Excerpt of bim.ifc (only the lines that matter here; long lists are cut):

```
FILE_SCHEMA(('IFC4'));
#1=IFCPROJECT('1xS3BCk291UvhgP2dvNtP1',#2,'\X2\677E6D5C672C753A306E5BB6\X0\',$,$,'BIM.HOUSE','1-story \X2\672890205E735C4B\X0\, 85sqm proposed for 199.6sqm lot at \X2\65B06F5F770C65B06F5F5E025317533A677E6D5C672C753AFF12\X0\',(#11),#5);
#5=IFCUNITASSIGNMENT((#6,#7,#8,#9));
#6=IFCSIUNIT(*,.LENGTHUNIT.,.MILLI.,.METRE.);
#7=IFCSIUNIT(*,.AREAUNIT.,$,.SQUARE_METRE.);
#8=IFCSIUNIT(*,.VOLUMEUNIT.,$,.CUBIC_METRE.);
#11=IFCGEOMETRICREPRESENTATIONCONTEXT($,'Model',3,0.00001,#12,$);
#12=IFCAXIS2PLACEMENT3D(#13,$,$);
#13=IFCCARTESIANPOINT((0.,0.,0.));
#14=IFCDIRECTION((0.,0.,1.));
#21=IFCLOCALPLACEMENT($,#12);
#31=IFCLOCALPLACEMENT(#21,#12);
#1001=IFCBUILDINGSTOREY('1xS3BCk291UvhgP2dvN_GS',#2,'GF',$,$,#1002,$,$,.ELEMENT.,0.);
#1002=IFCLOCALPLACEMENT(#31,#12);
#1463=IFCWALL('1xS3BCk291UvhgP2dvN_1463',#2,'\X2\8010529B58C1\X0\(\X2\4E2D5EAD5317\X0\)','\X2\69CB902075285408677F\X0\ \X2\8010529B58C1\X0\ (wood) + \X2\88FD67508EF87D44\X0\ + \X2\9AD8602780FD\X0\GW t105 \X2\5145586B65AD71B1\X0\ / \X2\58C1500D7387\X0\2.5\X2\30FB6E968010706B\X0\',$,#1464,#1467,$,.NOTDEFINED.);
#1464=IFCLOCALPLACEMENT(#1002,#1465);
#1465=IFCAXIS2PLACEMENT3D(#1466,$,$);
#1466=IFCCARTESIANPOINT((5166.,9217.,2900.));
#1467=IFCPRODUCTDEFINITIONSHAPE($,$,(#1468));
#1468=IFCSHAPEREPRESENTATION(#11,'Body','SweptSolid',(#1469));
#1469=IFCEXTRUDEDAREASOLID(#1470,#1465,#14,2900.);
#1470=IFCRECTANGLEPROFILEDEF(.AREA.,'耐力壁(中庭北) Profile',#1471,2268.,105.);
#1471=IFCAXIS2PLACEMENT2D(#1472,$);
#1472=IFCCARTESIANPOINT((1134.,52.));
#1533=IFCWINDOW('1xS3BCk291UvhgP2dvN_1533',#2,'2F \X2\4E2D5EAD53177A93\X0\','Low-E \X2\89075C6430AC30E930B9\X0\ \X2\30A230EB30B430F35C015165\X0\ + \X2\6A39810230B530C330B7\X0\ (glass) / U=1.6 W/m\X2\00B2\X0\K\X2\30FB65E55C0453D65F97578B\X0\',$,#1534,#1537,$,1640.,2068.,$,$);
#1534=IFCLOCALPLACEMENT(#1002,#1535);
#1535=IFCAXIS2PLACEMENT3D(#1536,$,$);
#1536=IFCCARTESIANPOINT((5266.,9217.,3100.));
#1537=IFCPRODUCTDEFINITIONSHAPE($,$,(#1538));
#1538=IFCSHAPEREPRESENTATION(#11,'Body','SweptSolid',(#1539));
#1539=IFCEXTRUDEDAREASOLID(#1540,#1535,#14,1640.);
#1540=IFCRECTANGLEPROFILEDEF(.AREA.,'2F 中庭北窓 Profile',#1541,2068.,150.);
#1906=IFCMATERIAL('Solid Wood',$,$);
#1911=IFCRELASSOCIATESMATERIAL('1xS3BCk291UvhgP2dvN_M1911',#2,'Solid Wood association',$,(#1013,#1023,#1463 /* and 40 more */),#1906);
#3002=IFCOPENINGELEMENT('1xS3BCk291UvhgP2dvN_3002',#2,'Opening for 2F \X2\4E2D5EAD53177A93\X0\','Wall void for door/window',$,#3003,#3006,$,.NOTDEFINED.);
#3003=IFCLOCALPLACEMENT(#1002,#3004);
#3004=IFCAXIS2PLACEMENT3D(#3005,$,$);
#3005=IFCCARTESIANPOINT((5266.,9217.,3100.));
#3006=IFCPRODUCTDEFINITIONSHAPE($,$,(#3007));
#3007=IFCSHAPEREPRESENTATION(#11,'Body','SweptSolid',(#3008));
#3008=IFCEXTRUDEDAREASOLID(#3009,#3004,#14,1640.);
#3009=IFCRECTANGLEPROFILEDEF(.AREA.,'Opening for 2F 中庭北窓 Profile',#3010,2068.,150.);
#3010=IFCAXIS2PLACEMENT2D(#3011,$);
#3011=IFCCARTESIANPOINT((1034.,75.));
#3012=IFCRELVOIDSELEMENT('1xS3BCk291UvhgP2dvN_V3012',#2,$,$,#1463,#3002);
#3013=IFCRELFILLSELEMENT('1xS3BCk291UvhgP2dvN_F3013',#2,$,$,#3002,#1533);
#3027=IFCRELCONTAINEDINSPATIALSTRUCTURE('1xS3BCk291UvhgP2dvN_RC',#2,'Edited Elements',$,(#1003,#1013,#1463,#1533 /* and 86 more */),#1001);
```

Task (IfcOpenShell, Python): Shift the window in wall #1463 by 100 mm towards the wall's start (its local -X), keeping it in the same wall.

```python
import ifcopenshell
import ifcopenshell.api.geometry
import ifcopenshell.util.placement
import ifcopenshell.util.unit

model = ifcopenshell.open("bim.ifc")
unit_scale = ifcopenshell.util.unit.calculate_unit_scale(model)

window = model.by_guid("1xS3BCk291UvhgP2dvN_1533")
opening = window.FillsVoids[0].RelatingOpeningElement
wall = opening.VoidsElements[0].RelatingBuildingElement

wall_matrix = ifcopenshell.util.placement.get_local_placement(wall.ObjectPlacement)
shift = wall_matrix[:3, 0] * -0.1 / unit_scale
before = ifcopenshell.util.placement.get_local_placement(window.ObjectPlacement)[:3, 3].copy()

# The window is not placed relative to its opening, so move both.
for product in (opening, window):
    matrix = ifcopenshell.util.placement.get_local_placement(product.ObjectPlacement)
    matrix[:3, 3] += shift
    ifcopenshell.api.geometry.edit_object_placement(model, product=product, matrix=matrix, is_si=False)

after = ifcopenshell.util.placement.get_local_placement(window.ObjectPlacement)[:3, 3]
print("window moved by", (after - before).round(3) + 0.0)

model.write("bim_edited.ifc")
```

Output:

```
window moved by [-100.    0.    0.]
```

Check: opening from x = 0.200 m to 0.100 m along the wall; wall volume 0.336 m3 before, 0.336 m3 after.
